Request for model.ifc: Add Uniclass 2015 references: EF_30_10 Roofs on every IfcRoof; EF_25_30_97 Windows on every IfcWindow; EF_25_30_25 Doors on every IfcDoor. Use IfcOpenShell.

First a look at what the model holds.

```python
import ifcopenshell

model = ifcopenshell.open("model.ifc")
print(model.schema)
print("classifications:", [c.Name for c in model.by_type("IfcClassification")])
for ifc_class in ("IfcDoor", "IfcRoof", "IfcStair", "IfcWall", "IfcWindow"):
    print(ifc_class, len(model.by_type(ifc_class)))
```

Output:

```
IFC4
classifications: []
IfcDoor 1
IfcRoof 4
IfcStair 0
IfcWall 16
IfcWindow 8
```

```python
import ifcopenshell
import ifcopenshell.api.classification

model = ifcopenshell.open("model.ifc")

system = ifcopenshell.api.classification.add_classification(model, classification="Uniclass 2015")

codes = {
    "IfcRoof": ("EF_30_10", "Roofs"),
    "IfcWindow": ("EF_25_30_97", "Windows"),
    "IfcDoor": ("EF_25_30_25", "Doors"),
}
for ifc_class, (code, name) in codes.items():
    products = model.by_type(ifc_class)
    ifcopenshell.api.classification.add_reference(
        model, products=products, classification=system, identification=code, name=name
    )
    print(code, len(products))

model.write("model_v2.ifc")
```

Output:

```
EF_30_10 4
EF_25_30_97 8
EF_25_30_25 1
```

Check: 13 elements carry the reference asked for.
